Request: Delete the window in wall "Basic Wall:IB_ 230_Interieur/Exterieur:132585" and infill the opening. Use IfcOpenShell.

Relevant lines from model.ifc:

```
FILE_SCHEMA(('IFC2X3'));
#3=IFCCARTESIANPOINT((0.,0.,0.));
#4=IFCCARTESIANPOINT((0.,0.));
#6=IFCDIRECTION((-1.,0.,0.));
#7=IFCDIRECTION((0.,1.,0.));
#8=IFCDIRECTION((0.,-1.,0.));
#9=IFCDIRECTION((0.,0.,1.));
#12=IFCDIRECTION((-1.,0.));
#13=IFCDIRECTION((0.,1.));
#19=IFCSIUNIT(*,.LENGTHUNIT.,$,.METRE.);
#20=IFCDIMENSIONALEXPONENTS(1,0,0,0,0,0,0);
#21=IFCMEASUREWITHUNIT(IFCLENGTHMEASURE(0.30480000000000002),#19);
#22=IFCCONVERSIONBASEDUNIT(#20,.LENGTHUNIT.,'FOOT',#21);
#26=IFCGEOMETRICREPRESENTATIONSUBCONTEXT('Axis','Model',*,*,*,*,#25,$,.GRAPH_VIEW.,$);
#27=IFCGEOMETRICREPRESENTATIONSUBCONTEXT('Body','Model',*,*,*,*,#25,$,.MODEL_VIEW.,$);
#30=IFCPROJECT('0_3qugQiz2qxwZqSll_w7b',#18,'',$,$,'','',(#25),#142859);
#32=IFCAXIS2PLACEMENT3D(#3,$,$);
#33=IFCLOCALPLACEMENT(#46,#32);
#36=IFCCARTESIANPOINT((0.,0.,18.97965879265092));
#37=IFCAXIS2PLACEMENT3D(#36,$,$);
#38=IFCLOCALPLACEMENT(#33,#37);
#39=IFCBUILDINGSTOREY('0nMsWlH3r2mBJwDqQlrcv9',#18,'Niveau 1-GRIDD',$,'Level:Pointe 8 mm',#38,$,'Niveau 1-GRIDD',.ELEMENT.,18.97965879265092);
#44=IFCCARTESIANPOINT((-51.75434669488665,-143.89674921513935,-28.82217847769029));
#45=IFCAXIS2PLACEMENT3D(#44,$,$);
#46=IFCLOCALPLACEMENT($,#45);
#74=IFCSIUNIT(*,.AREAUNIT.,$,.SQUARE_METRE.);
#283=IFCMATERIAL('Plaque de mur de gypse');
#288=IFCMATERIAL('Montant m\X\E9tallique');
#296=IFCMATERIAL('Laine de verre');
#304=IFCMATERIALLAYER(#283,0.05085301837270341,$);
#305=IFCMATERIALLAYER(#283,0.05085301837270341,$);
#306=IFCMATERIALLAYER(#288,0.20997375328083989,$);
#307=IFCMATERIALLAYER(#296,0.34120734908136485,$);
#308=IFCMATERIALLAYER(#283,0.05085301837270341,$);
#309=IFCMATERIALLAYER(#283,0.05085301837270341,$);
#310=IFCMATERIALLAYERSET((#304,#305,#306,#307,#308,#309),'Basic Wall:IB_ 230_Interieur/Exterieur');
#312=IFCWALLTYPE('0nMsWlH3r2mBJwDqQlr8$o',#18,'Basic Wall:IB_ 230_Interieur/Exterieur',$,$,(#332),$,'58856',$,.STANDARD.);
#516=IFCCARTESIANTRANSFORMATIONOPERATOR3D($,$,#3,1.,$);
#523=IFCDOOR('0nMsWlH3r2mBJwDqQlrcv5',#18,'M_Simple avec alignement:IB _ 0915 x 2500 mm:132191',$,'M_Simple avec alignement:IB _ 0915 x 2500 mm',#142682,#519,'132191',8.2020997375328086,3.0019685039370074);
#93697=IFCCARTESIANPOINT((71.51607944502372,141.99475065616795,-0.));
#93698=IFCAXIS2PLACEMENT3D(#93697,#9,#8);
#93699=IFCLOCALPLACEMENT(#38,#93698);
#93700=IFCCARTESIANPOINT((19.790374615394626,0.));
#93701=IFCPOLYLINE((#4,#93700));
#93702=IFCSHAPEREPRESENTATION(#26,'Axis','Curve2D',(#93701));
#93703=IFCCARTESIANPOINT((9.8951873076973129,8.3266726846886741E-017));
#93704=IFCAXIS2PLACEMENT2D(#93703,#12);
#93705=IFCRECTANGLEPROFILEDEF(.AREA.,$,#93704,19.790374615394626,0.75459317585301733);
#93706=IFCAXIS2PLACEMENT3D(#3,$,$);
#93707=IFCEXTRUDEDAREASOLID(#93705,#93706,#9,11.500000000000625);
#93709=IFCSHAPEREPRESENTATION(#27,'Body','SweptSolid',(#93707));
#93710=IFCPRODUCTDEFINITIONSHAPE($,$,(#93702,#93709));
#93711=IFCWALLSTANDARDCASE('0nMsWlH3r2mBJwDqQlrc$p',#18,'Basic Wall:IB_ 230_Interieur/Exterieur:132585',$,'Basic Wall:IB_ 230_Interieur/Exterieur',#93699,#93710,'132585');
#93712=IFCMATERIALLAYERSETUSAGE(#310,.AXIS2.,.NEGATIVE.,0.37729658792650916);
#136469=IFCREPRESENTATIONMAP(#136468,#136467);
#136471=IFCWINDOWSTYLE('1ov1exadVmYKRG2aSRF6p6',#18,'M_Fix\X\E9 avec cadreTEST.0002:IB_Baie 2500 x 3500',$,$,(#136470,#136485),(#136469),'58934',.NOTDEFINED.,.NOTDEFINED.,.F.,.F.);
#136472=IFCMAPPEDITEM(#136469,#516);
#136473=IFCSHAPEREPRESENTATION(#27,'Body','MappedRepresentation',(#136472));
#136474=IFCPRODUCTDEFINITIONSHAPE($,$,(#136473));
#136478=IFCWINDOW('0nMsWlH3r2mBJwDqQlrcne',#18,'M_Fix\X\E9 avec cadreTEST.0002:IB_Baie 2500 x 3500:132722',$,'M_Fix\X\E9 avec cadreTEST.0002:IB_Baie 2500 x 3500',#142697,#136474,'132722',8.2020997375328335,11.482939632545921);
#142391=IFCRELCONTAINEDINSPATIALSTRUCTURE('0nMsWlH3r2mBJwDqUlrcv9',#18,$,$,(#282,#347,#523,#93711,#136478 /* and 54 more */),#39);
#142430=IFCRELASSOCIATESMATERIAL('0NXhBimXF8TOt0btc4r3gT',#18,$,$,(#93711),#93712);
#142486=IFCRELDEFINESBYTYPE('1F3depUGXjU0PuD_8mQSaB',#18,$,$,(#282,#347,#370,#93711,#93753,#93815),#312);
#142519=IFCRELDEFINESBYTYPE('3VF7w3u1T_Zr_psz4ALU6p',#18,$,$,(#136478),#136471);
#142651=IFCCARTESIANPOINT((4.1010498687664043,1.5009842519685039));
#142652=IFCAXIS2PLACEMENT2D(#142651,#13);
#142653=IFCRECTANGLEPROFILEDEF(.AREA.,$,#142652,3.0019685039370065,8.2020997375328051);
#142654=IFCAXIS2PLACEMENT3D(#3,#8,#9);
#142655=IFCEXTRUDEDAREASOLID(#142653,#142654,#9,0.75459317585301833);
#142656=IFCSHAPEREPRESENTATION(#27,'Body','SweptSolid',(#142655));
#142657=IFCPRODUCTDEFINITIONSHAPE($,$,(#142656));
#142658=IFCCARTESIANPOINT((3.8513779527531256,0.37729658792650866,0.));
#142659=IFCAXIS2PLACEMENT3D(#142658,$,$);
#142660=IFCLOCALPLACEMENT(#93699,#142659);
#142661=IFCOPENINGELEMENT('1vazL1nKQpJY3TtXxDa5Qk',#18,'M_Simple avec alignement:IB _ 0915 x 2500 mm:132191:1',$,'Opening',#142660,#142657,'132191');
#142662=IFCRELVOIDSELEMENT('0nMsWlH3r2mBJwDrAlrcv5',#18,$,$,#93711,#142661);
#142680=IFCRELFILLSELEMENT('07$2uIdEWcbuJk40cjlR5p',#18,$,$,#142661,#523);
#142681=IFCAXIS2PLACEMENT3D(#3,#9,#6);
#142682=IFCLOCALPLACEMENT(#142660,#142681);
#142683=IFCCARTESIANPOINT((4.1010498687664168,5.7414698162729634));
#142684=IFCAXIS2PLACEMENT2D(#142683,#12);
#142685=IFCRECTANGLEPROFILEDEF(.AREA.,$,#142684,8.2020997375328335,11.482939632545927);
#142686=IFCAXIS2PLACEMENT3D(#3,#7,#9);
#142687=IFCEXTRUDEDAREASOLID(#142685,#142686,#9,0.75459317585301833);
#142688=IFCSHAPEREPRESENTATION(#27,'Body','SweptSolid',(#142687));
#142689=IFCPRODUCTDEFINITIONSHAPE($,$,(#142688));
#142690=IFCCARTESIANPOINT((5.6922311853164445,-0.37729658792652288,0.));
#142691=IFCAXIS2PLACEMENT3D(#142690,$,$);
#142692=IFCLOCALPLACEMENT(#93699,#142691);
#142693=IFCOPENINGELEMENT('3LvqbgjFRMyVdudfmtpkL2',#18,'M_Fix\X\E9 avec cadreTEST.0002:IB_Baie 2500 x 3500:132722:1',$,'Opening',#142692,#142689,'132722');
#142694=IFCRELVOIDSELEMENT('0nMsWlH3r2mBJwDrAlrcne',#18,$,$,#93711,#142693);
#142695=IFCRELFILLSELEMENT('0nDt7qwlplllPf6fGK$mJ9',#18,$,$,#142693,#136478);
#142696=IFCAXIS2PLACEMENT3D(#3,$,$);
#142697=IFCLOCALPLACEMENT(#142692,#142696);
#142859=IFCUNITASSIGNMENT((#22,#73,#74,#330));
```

```python
import ifcopenshell
import ifcopenshell.api.feature
import ifcopenshell.api.root
import ifcopenshell.geom
import ifcopenshell.util.shape

model = ifcopenshell.open("model.ifc")
settings = ifcopenshell.geom.settings()


def volume(element):
    """Net volume in cubic metres, openings subtracted."""
    shape = ifcopenshell.geom.create_shape(settings, element)
    return ifcopenshell.util.shape.get_volume(shape.geometry)


window = model.by_guid("0nMsWlH3r2mBJwDqQlrcne")
opening = window.FillsVoids[0].RelatingOpeningElement
wall = opening.VoidsElements[0].RelatingBuildingElement
before = volume(wall)

ifcopenshell.api.root.remove_product(model, product=window)
ifcopenshell.api.feature.remove_feature(model, feature=opening)

after = volume(wall)

print(f"wall volume {before:.3f} -> {after:.3f} m3")

model.write("model_updated.ifc")
```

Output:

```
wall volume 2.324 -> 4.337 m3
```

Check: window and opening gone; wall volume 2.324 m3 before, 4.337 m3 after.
